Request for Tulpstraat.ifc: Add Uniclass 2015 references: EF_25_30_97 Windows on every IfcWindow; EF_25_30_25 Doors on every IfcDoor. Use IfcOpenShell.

First a look at what the model holds.

```python
import ifcopenshell

model = ifcopenshell.open("Tulpstraat.ifc")
print(model.schema)
print("classifications:", [c.Name for c in model.by_type("IfcClassification")])
for ifc_class in ("IfcDoor", "IfcRoof", "IfcStair", "IfcWall", "IfcWindow"):
    print(ifc_class, len(model.by_type(ifc_class)))
```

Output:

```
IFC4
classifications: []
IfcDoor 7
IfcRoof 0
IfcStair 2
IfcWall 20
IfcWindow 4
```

```python
import ifcopenshell
import ifcopenshell.api.classification

model = ifcopenshell.open("Tulpstraat.ifc")

system = ifcopenshell.api.classification.add_classification(model, classification="Uniclass 2015")

codes = {
    "IfcWindow": ("EF_25_30_97", "Windows"),
    "IfcDoor": ("EF_25_30_25", "Doors"),
}
for ifc_class, (code, name) in codes.items():
    products = model.by_type(ifc_class)
    ifcopenshell.api.classification.add_reference(
        model, products=products, classification=system, identification=code, name=name
    )
    print(code, len(products))

model.write("Tulpstraat_updated.ifc")
```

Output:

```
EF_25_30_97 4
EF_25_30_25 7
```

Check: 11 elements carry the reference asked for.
